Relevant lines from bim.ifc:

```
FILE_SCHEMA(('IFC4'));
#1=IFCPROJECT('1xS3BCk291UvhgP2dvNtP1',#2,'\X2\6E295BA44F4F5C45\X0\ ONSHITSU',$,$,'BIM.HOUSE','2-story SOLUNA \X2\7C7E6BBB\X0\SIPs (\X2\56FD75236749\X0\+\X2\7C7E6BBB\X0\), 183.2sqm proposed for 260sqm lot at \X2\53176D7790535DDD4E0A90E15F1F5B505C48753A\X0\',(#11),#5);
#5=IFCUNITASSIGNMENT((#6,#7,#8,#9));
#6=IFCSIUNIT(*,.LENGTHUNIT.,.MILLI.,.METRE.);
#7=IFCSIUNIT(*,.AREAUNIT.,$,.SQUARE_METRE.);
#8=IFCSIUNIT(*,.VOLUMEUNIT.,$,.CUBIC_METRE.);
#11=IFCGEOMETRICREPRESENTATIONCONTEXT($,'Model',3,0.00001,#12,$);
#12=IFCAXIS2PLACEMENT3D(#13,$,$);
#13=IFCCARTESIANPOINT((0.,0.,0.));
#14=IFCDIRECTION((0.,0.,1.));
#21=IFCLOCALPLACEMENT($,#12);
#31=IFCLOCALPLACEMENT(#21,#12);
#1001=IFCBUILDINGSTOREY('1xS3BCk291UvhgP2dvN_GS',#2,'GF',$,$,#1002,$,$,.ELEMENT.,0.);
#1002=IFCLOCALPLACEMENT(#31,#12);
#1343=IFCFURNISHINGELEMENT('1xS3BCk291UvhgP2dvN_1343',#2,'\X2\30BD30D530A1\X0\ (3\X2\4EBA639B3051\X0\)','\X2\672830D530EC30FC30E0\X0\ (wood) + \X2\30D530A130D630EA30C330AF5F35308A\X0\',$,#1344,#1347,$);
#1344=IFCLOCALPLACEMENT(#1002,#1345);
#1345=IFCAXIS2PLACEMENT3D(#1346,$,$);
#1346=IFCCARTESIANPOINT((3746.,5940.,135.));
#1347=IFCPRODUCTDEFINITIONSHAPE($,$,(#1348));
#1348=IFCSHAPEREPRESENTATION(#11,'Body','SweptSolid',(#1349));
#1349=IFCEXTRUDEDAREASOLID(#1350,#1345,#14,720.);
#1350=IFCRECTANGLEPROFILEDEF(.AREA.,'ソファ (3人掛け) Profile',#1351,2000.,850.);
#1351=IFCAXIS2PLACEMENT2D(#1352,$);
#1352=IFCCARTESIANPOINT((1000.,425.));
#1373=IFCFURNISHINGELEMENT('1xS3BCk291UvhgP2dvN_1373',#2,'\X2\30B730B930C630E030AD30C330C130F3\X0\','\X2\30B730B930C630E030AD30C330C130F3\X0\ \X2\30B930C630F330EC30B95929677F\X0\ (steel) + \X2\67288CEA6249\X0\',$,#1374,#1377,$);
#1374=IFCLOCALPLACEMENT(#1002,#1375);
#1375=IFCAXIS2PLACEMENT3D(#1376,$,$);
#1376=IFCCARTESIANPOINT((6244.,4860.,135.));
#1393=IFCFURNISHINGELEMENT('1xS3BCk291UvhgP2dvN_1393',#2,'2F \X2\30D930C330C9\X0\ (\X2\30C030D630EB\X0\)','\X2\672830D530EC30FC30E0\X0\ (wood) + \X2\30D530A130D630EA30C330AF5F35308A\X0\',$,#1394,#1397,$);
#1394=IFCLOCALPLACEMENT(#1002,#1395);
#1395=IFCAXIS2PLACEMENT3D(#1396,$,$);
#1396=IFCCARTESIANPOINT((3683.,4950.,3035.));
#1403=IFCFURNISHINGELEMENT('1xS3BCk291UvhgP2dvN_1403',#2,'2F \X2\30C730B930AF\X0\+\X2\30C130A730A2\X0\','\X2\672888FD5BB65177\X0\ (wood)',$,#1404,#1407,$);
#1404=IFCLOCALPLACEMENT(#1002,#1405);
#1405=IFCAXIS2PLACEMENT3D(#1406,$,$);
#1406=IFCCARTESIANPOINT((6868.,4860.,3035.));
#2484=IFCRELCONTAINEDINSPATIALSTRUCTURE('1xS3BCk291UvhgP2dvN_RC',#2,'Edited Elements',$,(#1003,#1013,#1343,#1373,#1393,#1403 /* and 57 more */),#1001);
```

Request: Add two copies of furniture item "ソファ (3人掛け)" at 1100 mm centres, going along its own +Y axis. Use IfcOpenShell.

```python
import ifcopenshell
import ifcopenshell.api.geometry
import ifcopenshell.api.root
import ifcopenshell.util.element
import ifcopenshell.util.placement
import ifcopenshell.util.unit

model = ifcopenshell.open("bim.ifc")
unit_scale = ifcopenshell.util.unit.calculate_unit_scale(model)


def reuse_history(source, copy):
    """copy_class also copies each property set's owner history, people and application; keep the originals."""
    for rel in copy.IsDefinedBy:
        if rel.is_a("IfcRelDefinesByProperties") and (history := rel.RelatingPropertyDefinition.OwnerHistory):
            rel.RelatingPropertyDefinition.OwnerHistory = source.OwnerHistory
            ifcopenshell.util.element.remove_deep2(model, history)


source = model.by_guid("1xS3BCk291UvhgP2dvN_1343")
base = ifcopenshell.util.placement.get_local_placement(source.ObjectPlacement)
step = base[:3, 1] * 1.1 / unit_scale

for i in range(1, 3):
    copy = ifcopenshell.api.root.copy_class(model, product=source)
    copy.Representation = ifcopenshell.util.element.copy_deep(
        model, source.Representation, exclude=["IfcGeometricRepresentationContext", "IfcRepresentationMap"]
    )
    reuse_history(source, copy)
    matrix = base.copy()
    matrix[:3, 3] += i * step
    print("added at", matrix[:3, 3].round(3) + 0.0)
    ifcopenshell.api.geometry.edit_object_placement(model, product=copy, matrix=matrix, is_si=False)

model.write("bim_edited.ifc")
```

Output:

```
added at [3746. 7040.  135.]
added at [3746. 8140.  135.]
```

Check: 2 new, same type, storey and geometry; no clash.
